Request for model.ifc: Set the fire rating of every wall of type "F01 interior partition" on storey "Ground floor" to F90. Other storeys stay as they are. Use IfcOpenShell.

First a look at what the model holds.

```python
import ifcopenshell
import ifcopenshell.util.element

model = ifcopenshell.open("model.ifc")
print(model.schema)
storey = next(s for s in model.by_type("IfcBuildingStorey") if s.Name == "Ground floor")
walls = [e for e in ifcopenshell.util.element.get_decomposition(storey) if e.is_a("IfcWall")]
seen = {}
for e in walls:
    element_type = ifcopenshell.util.element.get_type(e)
    key = (element_type.Name if element_type != e and element_type else None, ifcopenshell.util.element.get_pset(e, "Pset_WallCommon", "FireRating"))
    seen[key] = seen.get(key, 0) + 1
for (name, value), count in sorted(seen.items(), key=str):
    print(count, "x", name, "|", value)
```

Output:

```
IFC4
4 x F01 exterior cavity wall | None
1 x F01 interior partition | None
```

```python
import ifcopenshell
import ifcopenshell.api.pset
import ifcopenshell.util.element

model = ifcopenshell.open("model.ifc")

storey = next(s for s in model.by_type("IfcBuildingStorey") if s.Name == "Ground floor")
walls = [e for e in ifcopenshell.util.element.get_decomposition(storey) if e.is_a("IfcWall")]

count = 0
for e in walls:
    element_type = ifcopenshell.util.element.get_type(e)
    if element_type in (None, e) or element_type.Name != "F01 interior partition":
        continue
    # add_pset returns the element's existing set when there is one.
    pset = ifcopenshell.api.pset.add_pset(model, product=e, name="Pset_WallCommon")
    ifcopenshell.api.pset.edit_pset(model, pset=pset, properties={"FireRating": "F90"})
    count += 1

print(count, "walls updated")

model.write("model-out.ifc")
```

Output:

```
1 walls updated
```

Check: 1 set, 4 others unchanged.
